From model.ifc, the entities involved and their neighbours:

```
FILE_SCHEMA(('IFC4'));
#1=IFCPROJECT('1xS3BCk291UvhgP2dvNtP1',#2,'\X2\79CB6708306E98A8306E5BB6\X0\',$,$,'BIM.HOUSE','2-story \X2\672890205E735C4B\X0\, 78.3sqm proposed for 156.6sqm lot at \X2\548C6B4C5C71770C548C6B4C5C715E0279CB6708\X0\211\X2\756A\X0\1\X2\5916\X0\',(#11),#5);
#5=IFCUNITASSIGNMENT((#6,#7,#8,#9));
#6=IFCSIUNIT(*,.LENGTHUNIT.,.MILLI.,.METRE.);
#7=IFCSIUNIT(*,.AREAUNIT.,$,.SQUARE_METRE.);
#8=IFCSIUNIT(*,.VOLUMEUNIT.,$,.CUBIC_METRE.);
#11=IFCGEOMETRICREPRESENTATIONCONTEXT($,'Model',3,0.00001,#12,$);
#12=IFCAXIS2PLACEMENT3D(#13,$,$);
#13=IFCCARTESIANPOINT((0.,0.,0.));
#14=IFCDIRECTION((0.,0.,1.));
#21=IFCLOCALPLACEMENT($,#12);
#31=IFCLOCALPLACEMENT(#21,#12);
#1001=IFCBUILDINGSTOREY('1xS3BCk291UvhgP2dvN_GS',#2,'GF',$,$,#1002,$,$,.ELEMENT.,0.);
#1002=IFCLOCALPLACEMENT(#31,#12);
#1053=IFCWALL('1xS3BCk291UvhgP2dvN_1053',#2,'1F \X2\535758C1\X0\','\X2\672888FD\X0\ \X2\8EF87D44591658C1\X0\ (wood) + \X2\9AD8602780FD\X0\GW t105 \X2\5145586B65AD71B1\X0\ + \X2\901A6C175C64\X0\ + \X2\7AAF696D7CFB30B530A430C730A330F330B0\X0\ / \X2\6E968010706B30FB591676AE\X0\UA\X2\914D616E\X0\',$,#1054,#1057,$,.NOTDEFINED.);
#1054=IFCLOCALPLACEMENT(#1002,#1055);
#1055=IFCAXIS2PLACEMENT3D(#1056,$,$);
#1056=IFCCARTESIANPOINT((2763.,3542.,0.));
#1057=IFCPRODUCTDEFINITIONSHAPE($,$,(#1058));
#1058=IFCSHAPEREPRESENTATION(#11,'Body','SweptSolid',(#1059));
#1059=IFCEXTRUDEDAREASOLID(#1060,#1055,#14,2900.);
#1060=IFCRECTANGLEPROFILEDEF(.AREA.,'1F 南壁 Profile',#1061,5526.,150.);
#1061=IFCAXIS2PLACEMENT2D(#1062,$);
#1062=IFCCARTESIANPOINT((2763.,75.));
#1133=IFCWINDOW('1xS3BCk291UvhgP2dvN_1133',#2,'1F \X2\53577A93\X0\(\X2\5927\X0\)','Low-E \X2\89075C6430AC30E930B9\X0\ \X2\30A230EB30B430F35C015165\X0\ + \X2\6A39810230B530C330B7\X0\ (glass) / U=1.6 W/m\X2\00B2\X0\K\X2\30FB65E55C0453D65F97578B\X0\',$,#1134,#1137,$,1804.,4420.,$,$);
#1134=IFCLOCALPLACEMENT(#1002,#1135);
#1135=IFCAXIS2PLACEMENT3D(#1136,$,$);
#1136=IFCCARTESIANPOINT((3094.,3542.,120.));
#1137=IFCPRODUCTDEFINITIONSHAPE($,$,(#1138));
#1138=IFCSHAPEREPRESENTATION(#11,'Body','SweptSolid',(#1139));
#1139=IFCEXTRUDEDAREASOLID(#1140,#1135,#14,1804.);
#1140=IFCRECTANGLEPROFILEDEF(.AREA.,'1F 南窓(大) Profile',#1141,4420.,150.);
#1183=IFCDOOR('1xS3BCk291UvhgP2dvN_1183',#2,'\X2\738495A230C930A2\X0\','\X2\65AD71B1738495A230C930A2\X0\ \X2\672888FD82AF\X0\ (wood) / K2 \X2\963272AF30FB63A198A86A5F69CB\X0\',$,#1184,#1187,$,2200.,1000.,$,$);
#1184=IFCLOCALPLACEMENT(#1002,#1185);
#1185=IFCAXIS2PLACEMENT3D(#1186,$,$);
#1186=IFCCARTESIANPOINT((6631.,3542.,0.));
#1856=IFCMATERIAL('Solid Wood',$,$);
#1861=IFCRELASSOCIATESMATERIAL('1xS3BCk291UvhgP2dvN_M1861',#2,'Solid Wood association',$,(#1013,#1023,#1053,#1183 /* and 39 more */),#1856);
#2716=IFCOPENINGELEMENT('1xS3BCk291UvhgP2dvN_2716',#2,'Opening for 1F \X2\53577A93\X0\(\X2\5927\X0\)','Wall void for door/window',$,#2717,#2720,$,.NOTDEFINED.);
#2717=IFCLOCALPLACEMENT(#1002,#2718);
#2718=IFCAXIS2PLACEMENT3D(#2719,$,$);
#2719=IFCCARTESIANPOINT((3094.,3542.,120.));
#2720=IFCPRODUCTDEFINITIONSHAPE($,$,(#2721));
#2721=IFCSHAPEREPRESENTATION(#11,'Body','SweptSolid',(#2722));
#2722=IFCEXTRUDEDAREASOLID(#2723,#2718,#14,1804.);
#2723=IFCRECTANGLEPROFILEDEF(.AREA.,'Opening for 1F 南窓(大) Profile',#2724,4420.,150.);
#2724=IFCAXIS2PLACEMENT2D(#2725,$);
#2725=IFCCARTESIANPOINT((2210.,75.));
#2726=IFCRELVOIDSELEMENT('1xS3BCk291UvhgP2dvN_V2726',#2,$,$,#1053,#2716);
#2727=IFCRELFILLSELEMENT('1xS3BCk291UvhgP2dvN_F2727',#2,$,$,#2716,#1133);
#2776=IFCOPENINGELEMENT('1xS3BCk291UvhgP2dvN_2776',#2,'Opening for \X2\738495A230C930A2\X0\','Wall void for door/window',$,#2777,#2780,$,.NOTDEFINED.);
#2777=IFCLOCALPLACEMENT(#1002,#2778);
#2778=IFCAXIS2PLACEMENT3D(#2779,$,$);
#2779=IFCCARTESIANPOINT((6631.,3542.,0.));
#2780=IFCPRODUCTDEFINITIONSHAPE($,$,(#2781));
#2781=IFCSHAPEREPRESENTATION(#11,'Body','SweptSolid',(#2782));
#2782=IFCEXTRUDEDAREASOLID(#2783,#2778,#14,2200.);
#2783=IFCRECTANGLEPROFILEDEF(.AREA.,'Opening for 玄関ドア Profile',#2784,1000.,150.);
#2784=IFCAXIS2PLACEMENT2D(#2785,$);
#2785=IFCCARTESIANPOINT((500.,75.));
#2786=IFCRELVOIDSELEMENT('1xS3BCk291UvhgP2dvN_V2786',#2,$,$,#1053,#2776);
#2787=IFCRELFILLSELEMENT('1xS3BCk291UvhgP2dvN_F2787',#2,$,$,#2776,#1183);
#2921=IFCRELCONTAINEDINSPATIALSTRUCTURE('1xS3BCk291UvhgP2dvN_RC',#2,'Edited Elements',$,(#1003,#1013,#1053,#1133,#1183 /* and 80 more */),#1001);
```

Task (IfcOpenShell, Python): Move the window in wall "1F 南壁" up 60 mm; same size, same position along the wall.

```python
import numpy as np
import ifcopenshell
import ifcopenshell.api.geometry
import ifcopenshell.util.placement
import ifcopenshell.util.unit

model = ifcopenshell.open("model.ifc")
unit_scale = ifcopenshell.util.unit.calculate_unit_scale(model)

window = model.by_id(1133)
opening = window.FillsVoids[0].RelatingOpeningElement
dz = 0.06 / unit_scale

shift = np.array([0.0, 0.0, dz])
# The window is not placed relative to its opening, so move both.
for product in (opening, window):
    matrix = ifcopenshell.util.placement.get_local_placement(product.ObjectPlacement)
    matrix[:3, 3] += shift
    ifcopenshell.api.geometry.edit_object_placement(model, product=product, matrix=matrix, is_si=False)

print(f"moved by {dz * unit_scale:+.3f} m")

model.write("model_updated.ifc")
```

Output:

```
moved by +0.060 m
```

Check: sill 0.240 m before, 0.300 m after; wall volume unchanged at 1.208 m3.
